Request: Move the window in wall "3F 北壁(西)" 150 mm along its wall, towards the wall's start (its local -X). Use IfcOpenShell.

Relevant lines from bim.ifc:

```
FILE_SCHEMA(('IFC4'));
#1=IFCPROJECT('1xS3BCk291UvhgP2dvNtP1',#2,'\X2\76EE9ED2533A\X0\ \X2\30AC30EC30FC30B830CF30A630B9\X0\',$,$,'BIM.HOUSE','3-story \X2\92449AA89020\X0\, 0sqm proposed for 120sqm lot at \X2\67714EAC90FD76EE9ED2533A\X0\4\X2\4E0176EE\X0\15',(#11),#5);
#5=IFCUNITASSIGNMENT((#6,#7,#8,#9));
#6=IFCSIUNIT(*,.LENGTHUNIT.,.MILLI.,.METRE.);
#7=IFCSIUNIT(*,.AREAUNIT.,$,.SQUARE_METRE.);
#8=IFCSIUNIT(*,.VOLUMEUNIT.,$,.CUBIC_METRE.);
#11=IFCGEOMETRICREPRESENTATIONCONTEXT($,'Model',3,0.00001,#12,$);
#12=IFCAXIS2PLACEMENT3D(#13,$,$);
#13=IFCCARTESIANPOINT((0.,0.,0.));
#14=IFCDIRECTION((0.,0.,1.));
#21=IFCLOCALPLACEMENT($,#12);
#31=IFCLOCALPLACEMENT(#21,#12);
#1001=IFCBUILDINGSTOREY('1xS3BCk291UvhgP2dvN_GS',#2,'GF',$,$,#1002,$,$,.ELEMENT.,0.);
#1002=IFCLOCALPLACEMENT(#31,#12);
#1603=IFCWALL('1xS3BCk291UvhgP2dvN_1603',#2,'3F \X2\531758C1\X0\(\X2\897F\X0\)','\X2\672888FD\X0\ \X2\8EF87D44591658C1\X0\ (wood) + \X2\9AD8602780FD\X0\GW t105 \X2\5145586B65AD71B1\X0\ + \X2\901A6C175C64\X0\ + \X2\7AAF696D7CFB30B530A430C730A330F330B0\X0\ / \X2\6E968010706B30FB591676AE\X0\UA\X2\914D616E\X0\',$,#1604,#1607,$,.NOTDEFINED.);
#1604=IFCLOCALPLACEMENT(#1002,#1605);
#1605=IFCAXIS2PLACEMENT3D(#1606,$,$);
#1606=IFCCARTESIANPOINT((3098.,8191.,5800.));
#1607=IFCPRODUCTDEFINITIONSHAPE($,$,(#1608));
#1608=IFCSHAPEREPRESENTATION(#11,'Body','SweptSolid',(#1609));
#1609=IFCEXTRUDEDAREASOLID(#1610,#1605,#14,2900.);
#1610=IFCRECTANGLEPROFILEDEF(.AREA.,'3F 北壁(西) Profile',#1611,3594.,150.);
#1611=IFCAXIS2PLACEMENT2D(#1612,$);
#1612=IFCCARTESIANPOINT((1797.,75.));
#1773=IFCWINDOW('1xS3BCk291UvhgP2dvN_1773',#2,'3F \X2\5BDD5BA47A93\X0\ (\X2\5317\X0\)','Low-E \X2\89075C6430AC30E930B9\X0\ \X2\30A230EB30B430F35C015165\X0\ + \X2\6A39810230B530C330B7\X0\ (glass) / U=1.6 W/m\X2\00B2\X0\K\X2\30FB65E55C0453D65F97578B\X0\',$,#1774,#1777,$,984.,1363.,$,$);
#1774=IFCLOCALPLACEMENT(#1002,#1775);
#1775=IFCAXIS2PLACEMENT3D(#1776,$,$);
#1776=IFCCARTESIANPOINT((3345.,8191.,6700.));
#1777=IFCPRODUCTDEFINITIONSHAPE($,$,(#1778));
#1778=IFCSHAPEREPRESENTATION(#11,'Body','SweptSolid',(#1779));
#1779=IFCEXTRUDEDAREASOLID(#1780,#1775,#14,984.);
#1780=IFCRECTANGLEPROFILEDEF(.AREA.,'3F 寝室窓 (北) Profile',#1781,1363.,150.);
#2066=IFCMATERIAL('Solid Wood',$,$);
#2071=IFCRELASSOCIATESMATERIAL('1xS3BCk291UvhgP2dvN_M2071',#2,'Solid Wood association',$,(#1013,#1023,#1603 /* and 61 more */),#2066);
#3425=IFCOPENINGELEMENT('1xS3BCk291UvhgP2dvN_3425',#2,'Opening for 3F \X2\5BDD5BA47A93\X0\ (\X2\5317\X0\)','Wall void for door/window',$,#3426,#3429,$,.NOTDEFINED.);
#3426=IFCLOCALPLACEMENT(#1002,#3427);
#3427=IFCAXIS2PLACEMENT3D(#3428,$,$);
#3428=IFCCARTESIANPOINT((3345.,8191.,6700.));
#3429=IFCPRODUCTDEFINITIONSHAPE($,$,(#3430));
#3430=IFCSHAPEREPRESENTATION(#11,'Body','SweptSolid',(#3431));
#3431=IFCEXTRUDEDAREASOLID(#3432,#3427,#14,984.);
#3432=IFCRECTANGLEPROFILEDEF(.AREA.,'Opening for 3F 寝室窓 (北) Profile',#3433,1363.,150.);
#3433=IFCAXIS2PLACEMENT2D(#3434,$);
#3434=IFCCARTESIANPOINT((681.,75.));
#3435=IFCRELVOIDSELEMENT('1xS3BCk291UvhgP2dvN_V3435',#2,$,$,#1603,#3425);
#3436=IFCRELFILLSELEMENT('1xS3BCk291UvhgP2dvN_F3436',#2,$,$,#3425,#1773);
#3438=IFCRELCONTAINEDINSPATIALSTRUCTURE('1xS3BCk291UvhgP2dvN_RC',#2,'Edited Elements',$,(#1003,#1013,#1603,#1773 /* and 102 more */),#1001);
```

```python
import ifcopenshell
import ifcopenshell.api.geometry
import ifcopenshell.util.placement
import ifcopenshell.util.unit

model = ifcopenshell.open("bim.ifc")
unit_scale = ifcopenshell.util.unit.calculate_unit_scale(model)

window = model.by_id(1773)
opening = window.FillsVoids[0].RelatingOpeningElement
wall = opening.VoidsElements[0].RelatingBuildingElement

wall_matrix = ifcopenshell.util.placement.get_local_placement(wall.ObjectPlacement)
shift = wall_matrix[:3, 0] * -0.15 / unit_scale
before = ifcopenshell.util.placement.get_local_placement(window.ObjectPlacement)[:3, 3].copy()

# The window is not placed relative to its opening, so move both.
for product in (opening, window):
    matrix = ifcopenshell.util.placement.get_local_placement(product.ObjectPlacement)
    matrix[:3, 3] += shift
    ifcopenshell.api.geometry.edit_object_placement(model, product=product, matrix=matrix, is_si=False)

after = ifcopenshell.util.placement.get_local_placement(window.ObjectPlacement)[:3, 3]
print("window moved by", (after - before).round(3) + 0.0)

model.write("bim_v2.ifc")
```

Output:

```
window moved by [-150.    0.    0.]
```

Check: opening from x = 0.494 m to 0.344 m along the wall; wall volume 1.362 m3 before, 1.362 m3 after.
